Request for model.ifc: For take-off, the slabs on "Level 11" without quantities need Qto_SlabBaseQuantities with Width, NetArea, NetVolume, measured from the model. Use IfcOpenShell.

First a look at what the model holds.

```python
import ifcopenshell
import ifcopenshell.util.element
import ifcopenshell.util.unit

model = ifcopenshell.open("model.ifc")
print(model.schema)
for unit_type in ("LENGTHUNIT", "AREAUNIT", "VOLUMEUNIT"):
    print(unit_type, ifcopenshell.util.unit.calculate_unit_scale(model, unit_type))
storey = next(s for s in model.by_type("IfcBuildingStorey") if s.Name == "Level 11")
slabs = [e for e in ifcopenshell.util.element.get_decomposition(storey) if e.is_a("IfcSlab")]
for e in sorted(slabs, key=lambda e: e.id()):
    print(e.id(), e.is_a(), e.Name, list(ifcopenshell.util.element.get_psets(e, qtos_only=True)), sep=" | ")
```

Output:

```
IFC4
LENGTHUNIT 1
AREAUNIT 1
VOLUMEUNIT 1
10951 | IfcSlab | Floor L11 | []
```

```python
import ifcopenshell
import ifcopenshell.api.pset
import ifcopenshell.geom
import ifcopenshell.util.element
import ifcopenshell.util.shape
import ifcopenshell.util.unit

model = ifcopenshell.open("model.ifc")
unit_scale = ifcopenshell.util.unit.calculate_unit_scale(model)
area_scale = ifcopenshell.util.unit.calculate_unit_scale(model, "AREAUNIT")
volume_scale = ifcopenshell.util.unit.calculate_unit_scale(model, "VOLUMEUNIT")
settings = ifcopenshell.geom.settings()

storey = next(s for s in model.by_type("IfcBuildingStorey") if s.Name == "Level 11")
slabs = [e for e in ifcopenshell.util.element.get_decomposition(storey) if e.is_a("IfcSlab")]

for e in sorted(slabs, key=lambda e: e.id()):
    if ifcopenshell.util.element.get_psets(e, qtos_only=True, should_inherit=False):
        continue
    # Geometry comes back in metres, in the element's own axes.
    shape = ifcopenshell.geom.create_shape(settings, e)
    values = {
        "Width": ifcopenshell.util.shape.get_z(shape.geometry) / unit_scale,
        "NetArea": ifcopenshell.util.shape.get_footprint_area(shape.geometry) / area_scale,
        "NetVolume": ifcopenshell.util.shape.get_volume(shape.geometry) / volume_scale,
    }
    qto = ifcopenshell.api.pset.add_qto(model, product=e, name="Qto_SlabBaseQuantities")
    ifcopenshell.api.pset.edit_qto(model, qto=qto, properties=values)
    print(e.id(), {k: round(v, 3) for k, v in values.items()})

model.write("model_v2.ifc")
```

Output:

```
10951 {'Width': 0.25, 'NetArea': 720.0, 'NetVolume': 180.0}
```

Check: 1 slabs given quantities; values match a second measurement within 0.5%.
